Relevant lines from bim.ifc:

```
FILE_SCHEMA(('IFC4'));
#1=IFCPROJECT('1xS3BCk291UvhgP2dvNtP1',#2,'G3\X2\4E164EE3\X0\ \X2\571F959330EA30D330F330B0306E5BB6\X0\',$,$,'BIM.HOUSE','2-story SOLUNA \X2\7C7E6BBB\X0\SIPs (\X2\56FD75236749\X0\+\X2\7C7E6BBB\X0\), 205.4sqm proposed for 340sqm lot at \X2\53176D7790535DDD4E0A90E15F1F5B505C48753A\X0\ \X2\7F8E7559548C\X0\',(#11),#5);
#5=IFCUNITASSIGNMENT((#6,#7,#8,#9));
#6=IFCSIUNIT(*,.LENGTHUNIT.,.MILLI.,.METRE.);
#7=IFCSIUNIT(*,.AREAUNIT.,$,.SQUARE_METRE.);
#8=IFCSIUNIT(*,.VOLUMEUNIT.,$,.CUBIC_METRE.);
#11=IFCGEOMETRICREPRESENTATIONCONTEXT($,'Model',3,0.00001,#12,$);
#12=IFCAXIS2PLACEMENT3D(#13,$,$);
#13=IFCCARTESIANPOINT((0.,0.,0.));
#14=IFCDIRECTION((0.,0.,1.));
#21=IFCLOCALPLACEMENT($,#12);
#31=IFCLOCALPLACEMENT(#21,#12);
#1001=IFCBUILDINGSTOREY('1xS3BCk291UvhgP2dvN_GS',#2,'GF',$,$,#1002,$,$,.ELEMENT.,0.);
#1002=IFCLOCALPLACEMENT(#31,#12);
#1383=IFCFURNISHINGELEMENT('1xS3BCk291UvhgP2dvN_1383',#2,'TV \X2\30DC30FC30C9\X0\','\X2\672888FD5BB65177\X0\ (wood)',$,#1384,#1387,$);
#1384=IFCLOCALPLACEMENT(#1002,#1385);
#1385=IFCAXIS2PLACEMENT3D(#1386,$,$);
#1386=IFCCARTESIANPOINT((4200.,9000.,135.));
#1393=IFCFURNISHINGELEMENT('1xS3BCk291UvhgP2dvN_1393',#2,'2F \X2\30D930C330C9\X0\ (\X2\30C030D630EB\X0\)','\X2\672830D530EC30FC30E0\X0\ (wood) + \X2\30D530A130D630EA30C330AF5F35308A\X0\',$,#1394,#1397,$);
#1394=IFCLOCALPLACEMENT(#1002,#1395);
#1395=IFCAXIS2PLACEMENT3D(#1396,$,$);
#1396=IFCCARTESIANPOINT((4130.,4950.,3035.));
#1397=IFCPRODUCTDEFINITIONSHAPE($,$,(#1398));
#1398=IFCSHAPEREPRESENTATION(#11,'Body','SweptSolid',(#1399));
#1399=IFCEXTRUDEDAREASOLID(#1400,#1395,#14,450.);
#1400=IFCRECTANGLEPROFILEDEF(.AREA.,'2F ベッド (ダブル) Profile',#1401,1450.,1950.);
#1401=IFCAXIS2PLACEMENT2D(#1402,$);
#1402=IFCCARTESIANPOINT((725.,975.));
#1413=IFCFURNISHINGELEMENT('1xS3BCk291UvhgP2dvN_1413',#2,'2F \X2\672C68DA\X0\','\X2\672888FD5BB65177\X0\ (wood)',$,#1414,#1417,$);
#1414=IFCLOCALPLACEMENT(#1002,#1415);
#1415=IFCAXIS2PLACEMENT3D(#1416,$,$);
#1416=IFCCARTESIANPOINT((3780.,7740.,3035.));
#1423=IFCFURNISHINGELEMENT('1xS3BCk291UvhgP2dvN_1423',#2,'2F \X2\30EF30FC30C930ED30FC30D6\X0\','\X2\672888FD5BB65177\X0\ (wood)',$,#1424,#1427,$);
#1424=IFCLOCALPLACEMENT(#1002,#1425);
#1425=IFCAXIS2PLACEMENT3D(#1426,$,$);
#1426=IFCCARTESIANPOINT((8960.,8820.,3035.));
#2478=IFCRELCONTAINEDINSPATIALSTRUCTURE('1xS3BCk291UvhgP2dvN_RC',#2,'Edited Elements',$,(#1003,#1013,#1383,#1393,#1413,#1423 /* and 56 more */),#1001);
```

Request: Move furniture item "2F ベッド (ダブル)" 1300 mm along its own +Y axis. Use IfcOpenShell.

```python
import ifcopenshell
import ifcopenshell.api.geometry
import ifcopenshell.util.placement

model = ifcopenshell.open("bim.ifc")

item = model.by_guid("1xS3BCk291UvhgP2dvN_1393")
matrix = ifcopenshell.util.placement.get_local_placement(item.ObjectPlacement)
matrix[:3, 3] += matrix[:3, 1] * 1300.0
ifcopenshell.api.geometry.edit_object_placement(model, product=item, matrix=matrix, is_si=False)

print(ifcopenshell.util.placement.get_local_placement(item.ObjectPlacement).round(3) + 0.0)

model.write("bim_v2.ifc")
```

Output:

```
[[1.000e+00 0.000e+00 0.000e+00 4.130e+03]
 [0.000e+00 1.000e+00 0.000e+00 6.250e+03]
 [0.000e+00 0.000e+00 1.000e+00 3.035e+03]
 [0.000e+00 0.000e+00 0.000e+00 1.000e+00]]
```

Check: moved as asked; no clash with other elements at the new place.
